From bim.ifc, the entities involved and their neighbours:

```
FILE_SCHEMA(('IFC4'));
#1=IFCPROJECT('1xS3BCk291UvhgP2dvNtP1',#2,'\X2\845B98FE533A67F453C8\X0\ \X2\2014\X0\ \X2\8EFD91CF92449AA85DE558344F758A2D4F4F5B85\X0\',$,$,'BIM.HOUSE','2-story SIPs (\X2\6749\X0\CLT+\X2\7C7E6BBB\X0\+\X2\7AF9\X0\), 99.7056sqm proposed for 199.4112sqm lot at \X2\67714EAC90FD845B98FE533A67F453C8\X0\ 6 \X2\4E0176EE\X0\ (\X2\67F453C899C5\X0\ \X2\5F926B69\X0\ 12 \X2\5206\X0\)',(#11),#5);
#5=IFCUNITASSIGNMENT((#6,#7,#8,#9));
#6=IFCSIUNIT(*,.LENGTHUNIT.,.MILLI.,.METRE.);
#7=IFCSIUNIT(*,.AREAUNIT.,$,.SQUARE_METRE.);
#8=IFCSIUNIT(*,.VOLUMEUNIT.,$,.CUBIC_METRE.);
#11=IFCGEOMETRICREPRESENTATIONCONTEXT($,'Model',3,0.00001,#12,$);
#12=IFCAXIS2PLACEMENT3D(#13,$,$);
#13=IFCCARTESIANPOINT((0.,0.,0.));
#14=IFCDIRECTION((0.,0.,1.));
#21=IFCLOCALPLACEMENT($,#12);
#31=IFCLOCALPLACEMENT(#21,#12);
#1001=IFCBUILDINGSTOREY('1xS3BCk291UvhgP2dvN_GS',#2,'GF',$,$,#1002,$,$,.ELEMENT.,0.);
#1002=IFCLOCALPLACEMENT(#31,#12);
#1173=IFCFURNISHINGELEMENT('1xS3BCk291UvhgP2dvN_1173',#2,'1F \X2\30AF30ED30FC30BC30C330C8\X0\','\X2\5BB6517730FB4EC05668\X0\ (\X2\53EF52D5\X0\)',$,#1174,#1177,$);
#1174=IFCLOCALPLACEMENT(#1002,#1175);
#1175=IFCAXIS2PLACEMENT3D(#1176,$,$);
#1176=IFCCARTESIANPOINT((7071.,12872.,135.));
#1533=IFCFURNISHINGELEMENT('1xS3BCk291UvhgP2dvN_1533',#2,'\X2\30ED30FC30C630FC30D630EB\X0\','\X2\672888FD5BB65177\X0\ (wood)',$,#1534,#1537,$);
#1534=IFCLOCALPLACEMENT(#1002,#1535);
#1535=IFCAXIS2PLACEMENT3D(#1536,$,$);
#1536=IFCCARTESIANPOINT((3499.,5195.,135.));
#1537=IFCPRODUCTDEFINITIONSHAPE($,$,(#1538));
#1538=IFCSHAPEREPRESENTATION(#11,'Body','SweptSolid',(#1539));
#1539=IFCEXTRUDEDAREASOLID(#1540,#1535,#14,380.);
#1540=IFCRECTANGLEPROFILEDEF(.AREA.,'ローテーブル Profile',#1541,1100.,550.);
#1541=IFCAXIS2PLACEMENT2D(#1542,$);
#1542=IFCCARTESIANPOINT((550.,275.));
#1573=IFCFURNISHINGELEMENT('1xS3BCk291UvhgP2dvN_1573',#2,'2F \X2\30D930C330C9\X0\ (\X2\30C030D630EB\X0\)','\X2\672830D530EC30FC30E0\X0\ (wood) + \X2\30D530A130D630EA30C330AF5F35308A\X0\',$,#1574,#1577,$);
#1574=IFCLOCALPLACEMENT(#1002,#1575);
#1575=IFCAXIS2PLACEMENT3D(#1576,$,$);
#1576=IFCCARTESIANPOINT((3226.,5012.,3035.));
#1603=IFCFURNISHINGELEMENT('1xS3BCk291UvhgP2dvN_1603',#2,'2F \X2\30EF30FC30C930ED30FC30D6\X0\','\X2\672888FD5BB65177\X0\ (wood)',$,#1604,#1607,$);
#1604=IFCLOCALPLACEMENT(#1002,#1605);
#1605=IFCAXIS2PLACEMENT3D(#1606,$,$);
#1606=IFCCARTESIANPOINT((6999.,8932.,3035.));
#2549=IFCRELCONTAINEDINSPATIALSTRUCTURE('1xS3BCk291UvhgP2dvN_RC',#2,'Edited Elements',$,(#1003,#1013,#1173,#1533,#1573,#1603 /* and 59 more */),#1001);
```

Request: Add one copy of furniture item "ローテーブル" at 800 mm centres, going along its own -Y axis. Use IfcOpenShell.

```python
import ifcopenshell
import ifcopenshell.api.geometry
import ifcopenshell.api.root
import ifcopenshell.util.element
import ifcopenshell.util.placement
import ifcopenshell.util.unit

model = ifcopenshell.open("bim.ifc")
unit_scale = ifcopenshell.util.unit.calculate_unit_scale(model)


def reuse_history(source, copy):
    """copy_class also copies each property set's owner history, people and application; keep the originals."""
    for rel in copy.IsDefinedBy:
        if rel.is_a("IfcRelDefinesByProperties") and (history := rel.RelatingPropertyDefinition.OwnerHistory):
            rel.RelatingPropertyDefinition.OwnerHistory = source.OwnerHistory
            ifcopenshell.util.element.remove_deep2(model, history)


source = model.by_guid("1xS3BCk291UvhgP2dvN_1533")
base = ifcopenshell.util.placement.get_local_placement(source.ObjectPlacement)
step = -base[:3, 1] * 0.8 / unit_scale

for i in range(1, 2):
    copy = ifcopenshell.api.root.copy_class(model, product=source)
    copy.Representation = ifcopenshell.util.element.copy_deep(
        model, source.Representation, exclude=["IfcGeometricRepresentationContext", "IfcRepresentationMap"]
    )
    reuse_history(source, copy)
    matrix = base.copy()
    matrix[:3, 3] += i * step
    print("added at", matrix[:3, 3].round(3) + 0.0)
    ifcopenshell.api.geometry.edit_object_placement(model, product=copy, matrix=matrix, is_si=False)

model.write("bim_v2.ifc")
```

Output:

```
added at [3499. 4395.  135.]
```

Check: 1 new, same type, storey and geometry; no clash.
